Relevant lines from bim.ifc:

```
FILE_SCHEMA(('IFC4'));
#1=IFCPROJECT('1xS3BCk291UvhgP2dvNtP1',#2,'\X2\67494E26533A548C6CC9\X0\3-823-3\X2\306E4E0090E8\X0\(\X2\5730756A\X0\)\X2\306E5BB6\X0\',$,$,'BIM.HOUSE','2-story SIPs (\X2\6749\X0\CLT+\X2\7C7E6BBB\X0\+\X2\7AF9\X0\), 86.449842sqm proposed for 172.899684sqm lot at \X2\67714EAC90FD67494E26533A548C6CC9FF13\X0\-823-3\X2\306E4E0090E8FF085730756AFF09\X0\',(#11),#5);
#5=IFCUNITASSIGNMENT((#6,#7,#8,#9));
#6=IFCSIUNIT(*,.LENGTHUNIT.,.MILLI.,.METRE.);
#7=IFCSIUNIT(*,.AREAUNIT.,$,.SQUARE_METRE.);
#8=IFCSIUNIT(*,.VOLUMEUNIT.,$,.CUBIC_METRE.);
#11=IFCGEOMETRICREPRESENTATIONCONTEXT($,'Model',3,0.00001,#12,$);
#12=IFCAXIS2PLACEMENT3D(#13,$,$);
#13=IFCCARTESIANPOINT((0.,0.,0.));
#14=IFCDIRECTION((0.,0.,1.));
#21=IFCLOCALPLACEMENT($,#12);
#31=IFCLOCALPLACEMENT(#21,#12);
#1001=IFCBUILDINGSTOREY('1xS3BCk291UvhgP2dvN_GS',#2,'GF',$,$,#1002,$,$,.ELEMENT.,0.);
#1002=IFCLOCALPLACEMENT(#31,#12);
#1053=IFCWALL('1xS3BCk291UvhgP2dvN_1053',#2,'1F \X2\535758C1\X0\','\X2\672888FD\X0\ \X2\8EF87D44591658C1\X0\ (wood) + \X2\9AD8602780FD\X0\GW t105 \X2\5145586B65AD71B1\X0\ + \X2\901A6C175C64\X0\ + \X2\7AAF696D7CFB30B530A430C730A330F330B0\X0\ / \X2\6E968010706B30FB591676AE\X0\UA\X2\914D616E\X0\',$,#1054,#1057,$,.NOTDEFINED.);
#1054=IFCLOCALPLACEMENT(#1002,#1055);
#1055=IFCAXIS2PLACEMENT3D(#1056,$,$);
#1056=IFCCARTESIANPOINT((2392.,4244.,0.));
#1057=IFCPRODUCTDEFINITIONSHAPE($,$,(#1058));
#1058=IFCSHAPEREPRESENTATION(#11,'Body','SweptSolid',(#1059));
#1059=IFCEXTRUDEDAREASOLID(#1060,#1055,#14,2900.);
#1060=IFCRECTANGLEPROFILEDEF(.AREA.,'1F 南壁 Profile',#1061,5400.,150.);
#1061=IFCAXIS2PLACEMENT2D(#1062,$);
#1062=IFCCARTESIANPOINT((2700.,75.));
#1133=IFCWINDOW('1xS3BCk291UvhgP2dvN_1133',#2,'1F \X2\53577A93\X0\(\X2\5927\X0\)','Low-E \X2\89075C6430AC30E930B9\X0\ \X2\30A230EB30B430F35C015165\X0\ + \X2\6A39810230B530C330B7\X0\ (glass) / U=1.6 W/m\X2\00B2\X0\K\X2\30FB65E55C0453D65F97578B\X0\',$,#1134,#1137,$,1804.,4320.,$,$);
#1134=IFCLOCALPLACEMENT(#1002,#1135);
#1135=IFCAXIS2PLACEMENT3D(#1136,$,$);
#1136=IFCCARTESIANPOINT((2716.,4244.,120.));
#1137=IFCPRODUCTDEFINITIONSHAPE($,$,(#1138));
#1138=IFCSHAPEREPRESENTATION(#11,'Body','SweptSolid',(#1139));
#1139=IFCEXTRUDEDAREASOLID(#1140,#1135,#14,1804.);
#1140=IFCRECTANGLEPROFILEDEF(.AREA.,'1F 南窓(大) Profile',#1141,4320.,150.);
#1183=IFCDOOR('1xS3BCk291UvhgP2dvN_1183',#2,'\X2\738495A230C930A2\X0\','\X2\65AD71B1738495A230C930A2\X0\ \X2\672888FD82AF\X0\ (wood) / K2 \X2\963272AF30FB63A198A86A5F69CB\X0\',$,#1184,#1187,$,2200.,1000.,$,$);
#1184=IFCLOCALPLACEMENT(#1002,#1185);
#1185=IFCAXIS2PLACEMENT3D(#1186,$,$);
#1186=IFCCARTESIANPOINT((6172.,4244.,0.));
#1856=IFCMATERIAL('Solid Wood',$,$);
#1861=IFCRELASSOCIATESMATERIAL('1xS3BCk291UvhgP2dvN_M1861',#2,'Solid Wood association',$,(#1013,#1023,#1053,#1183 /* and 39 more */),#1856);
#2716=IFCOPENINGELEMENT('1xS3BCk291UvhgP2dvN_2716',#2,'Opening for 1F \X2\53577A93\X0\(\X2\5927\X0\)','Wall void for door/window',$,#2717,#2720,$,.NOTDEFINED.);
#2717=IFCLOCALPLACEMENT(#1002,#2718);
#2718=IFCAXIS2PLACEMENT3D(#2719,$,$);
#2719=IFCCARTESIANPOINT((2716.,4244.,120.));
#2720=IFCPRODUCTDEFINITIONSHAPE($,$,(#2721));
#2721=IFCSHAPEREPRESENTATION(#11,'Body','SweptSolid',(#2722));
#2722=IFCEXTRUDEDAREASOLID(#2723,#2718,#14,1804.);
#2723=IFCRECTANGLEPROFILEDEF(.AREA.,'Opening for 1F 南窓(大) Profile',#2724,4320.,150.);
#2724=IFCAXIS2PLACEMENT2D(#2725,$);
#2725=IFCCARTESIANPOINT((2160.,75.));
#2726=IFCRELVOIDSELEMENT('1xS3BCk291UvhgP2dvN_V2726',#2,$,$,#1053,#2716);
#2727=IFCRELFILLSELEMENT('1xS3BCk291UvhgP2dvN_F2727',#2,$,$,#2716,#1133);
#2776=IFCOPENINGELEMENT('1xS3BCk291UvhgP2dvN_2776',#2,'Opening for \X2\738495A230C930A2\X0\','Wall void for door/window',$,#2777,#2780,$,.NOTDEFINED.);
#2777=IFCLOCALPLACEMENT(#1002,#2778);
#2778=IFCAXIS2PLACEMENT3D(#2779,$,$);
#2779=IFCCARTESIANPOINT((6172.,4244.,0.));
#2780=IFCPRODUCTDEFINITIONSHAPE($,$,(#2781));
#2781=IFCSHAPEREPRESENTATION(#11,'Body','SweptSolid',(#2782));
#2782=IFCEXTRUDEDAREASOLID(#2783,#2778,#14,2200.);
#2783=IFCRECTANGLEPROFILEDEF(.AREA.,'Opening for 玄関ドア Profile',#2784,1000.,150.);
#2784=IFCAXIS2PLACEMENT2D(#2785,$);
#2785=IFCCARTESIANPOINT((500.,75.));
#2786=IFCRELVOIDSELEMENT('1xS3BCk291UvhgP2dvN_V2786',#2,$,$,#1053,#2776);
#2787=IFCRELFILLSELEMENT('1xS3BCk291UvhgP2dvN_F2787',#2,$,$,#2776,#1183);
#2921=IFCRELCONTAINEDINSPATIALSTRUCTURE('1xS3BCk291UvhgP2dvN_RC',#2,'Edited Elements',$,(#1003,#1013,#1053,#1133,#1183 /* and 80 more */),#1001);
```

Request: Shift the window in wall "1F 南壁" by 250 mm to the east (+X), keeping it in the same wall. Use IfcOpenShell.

```python
import ifcopenshell
import ifcopenshell.api.geometry
import ifcopenshell.util.placement
import ifcopenshell.util.unit

model = ifcopenshell.open("bim.ifc")
unit_scale = ifcopenshell.util.unit.calculate_unit_scale(model)

window = model.by_guid("1xS3BCk291UvhgP2dvN_1133")
opening = window.FillsVoids[0].RelatingOpeningElement
wall = opening.VoidsElements[0].RelatingBuildingElement

wall_matrix = ifcopenshell.util.placement.get_local_placement(wall.ObjectPlacement)
shift = wall_matrix[:3, 0] * 0.25 / unit_scale
before = ifcopenshell.util.placement.get_local_placement(window.ObjectPlacement)[:3, 3].copy()

# The window is not placed relative to its opening, so move both.
for product in (opening, window):
    matrix = ifcopenshell.util.placement.get_local_placement(product.ObjectPlacement)
    matrix[:3, 3] += shift
    ifcopenshell.api.geometry.edit_object_placement(model, product=product, matrix=matrix, is_si=False)

after = ifcopenshell.util.placement.get_local_placement(window.ObjectPlacement)[:3, 3]
print("window moved by", (after - before).round(3) + 0.0)

model.write("bim_rev.ifc")
```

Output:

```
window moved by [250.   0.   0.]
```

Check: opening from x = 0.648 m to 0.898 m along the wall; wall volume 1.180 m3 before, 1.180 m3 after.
